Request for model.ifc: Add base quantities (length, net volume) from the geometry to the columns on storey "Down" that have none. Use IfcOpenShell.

First a look at what the model holds.

```python
import ifcopenshell
import ifcopenshell.util.element
import ifcopenshell.util.unit

model = ifcopenshell.open("model.ifc")
print(model.schema)
for unit_type in ("LENGTHUNIT", "AREAUNIT", "VOLUMEUNIT"):
    print(unit_type, ifcopenshell.util.unit.calculate_unit_scale(model, unit_type))
storey = next(s for s in model.by_type("IfcBuildingStorey") if s.Name == "Down")
columns = [e for e in ifcopenshell.util.element.get_decomposition(storey) if e.is_a("IfcColumn")]
for e in sorted(columns, key=lambda e: e.id()):
    print(e.id(), e.is_a(), e.Name, list(ifcopenshell.util.element.get_psets(e, qtos_only=True)), sep=" | ")
```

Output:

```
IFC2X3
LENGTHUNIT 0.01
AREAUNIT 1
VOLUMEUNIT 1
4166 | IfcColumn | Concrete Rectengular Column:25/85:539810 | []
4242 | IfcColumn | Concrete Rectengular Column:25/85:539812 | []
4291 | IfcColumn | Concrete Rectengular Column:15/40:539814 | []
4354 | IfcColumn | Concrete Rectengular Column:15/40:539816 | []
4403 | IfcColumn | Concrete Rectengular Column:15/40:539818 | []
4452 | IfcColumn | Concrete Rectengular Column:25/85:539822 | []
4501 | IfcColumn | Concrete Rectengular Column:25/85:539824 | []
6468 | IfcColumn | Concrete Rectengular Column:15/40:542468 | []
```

```python
import ifcopenshell
import ifcopenshell.api.pset
import ifcopenshell.geom
import ifcopenshell.util.element
import ifcopenshell.util.shape
import ifcopenshell.util.unit

model = ifcopenshell.open("model.ifc")
unit_scale = ifcopenshell.util.unit.calculate_unit_scale(model)
volume_scale = ifcopenshell.util.unit.calculate_unit_scale(model, "VOLUMEUNIT")
settings = ifcopenshell.geom.settings()

storey = next(s for s in model.by_type("IfcBuildingStorey") if s.Name == "Down")
columns = [e for e in ifcopenshell.util.element.get_decomposition(storey) if e.is_a("IfcColumn")]

for e in sorted(columns, key=lambda e: e.id()):
    if ifcopenshell.util.element.get_psets(e, qtos_only=True, should_inherit=False):
        continue
    # Geometry comes back in metres, in the element's own axes.
    shape = ifcopenshell.geom.create_shape(settings, e)
    values = {
        "Length": ifcopenshell.util.shape.get_z(shape.geometry) / unit_scale,
        "NetVolume": ifcopenshell.util.shape.get_volume(shape.geometry) / volume_scale,
    }
    qto = ifcopenshell.api.pset.add_qto(model, product=e, name="BaseQuantities")
    ifcopenshell.api.pset.edit_qto(model, qto=qto, properties=values)
    print(e.id(), {k: round(v, 3) for k, v in values.items()})

model.write("model_edited.ifc")
```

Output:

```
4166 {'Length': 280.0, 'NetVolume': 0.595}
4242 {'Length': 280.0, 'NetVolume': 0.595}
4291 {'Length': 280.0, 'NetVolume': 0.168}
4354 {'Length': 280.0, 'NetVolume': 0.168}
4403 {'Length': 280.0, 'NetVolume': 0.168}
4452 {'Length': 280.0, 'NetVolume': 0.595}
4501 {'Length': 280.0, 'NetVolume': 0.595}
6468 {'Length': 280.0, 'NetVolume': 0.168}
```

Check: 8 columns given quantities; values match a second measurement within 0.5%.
